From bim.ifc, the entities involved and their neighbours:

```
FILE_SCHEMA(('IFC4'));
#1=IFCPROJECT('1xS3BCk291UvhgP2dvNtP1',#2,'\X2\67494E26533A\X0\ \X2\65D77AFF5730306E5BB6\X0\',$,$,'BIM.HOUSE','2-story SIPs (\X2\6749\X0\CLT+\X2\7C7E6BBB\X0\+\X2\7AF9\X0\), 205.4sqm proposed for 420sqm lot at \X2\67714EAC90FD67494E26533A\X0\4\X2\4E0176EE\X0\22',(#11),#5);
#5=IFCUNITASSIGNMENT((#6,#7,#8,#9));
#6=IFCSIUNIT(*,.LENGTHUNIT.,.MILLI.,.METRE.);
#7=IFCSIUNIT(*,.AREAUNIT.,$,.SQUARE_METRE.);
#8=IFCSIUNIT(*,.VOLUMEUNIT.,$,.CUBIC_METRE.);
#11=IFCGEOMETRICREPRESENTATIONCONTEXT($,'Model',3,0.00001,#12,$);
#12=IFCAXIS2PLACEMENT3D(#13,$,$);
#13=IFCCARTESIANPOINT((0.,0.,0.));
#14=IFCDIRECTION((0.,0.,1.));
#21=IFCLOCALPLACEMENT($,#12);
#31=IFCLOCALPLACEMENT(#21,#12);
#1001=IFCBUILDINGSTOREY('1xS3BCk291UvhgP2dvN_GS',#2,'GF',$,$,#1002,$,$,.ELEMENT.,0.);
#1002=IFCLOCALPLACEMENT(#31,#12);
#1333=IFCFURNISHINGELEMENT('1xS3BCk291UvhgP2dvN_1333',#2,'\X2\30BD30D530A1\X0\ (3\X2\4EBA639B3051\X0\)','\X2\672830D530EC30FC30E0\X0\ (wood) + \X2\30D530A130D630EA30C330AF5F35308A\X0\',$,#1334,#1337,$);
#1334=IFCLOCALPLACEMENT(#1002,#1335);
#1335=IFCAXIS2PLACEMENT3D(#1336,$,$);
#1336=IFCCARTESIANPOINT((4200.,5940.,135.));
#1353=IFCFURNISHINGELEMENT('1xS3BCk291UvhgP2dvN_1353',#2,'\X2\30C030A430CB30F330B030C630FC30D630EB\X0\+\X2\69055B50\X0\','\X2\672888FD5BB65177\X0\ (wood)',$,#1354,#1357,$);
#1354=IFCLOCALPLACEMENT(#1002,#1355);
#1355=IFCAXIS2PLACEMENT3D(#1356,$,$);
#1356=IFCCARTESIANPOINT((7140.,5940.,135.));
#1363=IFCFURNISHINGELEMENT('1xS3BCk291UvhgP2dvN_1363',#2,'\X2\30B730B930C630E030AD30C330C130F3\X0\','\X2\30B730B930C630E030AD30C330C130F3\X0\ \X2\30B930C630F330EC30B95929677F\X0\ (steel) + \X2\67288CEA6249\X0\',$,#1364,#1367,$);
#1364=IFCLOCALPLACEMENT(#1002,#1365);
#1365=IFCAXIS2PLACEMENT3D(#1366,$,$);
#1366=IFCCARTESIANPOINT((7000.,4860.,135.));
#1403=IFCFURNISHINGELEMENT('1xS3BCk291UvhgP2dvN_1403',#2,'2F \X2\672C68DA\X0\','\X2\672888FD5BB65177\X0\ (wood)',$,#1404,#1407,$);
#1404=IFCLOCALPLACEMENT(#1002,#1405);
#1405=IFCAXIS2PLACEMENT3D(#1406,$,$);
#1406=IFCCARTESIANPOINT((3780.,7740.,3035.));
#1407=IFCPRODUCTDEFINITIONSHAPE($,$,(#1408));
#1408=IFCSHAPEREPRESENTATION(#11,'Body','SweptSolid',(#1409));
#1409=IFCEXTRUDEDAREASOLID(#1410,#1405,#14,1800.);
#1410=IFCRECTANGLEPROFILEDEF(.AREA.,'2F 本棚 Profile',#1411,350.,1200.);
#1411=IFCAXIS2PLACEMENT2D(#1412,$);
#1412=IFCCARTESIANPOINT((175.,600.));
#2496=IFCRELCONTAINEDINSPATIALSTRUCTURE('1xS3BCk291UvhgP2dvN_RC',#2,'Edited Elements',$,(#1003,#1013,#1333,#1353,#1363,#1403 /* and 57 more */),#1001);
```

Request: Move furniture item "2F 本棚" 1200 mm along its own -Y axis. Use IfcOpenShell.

```python
import ifcopenshell
import ifcopenshell.api.geometry
import ifcopenshell.util.placement
import ifcopenshell.util.unit

model = ifcopenshell.open("bim.ifc")
unit_scale = ifcopenshell.util.unit.calculate_unit_scale(model)

item = model.by_guid("1xS3BCk291UvhgP2dvN_1403")
matrix = ifcopenshell.util.placement.get_local_placement(item.ObjectPlacement)
matrix[:3, 3] -= matrix[:3, 1] * 1.2 / unit_scale
ifcopenshell.api.geometry.edit_object_placement(model, product=item, matrix=matrix, is_si=False)

print(ifcopenshell.util.placement.get_local_placement(item.ObjectPlacement).round(3) + 0.0)

model.write("bim_updated.ifc")
```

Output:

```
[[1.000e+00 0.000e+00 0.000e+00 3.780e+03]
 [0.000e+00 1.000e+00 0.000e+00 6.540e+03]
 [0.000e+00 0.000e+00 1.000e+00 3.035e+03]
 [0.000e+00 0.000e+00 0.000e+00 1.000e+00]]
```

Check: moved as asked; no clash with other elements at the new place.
